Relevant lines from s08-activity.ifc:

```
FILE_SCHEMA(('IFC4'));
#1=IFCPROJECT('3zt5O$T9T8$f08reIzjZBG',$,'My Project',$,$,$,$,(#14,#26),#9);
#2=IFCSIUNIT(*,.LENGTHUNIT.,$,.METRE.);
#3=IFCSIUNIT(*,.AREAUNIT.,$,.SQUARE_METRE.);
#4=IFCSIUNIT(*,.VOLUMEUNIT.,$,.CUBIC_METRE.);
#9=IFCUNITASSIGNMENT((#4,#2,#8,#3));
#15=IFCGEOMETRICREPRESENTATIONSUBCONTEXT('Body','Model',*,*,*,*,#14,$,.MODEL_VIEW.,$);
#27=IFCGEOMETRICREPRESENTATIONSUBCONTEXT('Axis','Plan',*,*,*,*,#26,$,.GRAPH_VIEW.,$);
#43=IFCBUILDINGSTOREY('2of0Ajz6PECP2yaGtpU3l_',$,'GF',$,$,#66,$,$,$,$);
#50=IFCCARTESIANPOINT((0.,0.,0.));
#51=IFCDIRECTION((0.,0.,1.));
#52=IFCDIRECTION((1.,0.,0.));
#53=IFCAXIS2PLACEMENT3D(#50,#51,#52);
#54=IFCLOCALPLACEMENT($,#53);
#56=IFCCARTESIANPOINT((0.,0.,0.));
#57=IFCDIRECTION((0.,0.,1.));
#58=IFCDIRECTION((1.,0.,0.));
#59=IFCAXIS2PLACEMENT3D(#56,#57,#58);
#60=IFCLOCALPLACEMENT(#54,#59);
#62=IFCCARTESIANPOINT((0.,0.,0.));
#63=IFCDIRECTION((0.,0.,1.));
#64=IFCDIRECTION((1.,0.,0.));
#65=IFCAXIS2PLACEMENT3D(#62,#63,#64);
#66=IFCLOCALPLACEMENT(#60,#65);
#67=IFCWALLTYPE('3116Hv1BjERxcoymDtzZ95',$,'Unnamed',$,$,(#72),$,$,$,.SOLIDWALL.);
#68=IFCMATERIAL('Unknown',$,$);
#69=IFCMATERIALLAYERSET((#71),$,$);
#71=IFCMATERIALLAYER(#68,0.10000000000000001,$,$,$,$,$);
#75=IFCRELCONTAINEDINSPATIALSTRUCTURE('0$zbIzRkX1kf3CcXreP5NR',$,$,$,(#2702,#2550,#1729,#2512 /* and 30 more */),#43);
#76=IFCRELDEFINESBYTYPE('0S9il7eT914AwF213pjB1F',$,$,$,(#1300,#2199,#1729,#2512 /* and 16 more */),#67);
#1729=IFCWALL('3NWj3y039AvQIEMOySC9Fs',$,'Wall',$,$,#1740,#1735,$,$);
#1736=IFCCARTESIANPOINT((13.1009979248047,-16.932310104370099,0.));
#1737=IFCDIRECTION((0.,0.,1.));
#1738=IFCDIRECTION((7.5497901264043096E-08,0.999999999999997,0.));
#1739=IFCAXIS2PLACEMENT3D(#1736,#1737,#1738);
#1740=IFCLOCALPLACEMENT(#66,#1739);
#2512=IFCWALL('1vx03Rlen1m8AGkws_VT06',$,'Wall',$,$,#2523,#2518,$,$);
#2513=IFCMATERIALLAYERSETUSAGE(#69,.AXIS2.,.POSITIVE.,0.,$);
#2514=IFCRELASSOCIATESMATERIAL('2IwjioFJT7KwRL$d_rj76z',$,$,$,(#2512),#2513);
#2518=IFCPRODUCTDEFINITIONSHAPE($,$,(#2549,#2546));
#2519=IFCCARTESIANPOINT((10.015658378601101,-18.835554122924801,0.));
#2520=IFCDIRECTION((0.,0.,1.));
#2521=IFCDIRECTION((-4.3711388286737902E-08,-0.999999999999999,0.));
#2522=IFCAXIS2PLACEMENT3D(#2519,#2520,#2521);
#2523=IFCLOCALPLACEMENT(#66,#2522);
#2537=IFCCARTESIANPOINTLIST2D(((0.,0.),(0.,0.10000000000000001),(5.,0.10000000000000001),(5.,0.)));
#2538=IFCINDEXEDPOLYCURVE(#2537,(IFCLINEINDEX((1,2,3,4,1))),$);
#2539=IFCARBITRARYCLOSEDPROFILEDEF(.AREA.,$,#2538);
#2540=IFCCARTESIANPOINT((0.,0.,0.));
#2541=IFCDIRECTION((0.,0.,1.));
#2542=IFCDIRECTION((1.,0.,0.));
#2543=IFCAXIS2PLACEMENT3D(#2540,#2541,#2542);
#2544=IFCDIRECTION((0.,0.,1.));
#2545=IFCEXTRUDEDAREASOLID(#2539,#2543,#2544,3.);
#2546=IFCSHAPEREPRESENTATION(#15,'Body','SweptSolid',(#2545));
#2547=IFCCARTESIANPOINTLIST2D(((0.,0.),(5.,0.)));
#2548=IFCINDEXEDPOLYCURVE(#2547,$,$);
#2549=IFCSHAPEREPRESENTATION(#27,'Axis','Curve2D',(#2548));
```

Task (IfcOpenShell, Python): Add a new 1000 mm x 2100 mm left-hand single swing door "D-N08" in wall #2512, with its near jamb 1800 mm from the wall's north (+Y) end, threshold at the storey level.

```python
import numpy as np
import ifcopenshell
import ifcopenshell.api.feature
import ifcopenshell.api.geometry
import ifcopenshell.api.root
import ifcopenshell.api.spatial
import ifcopenshell.geom
import ifcopenshell.util.element
import ifcopenshell.util.placement
import ifcopenshell.util.representation
import ifcopenshell.util.shape
import ifcopenshell.util.unit

model = ifcopenshell.open("s08-activity.ifc")
unit_scale = ifcopenshell.util.unit.calculate_unit_scale(model)
settings = ifcopenshell.geom.settings()


def volume(element):
    """Net volume in cubic metres, openings subtracted."""
    shape = ifcopenshell.geom.create_shape(settings, element)
    return ifcopenshell.util.shape.get_volume(shape.geometry)


wall = model.by_guid("1vx03Rlen1m8AGkws_VT06")
storey = ifcopenshell.util.element.get_container(wall, ifc_class="IfcBuildingStorey")
context = ifcopenshell.util.representation.get_context(model, "Model", "Body", "MODEL_VIEW")
before = volume(wall)

width, height, from_end, sill = 1, 2.1, 1.8, 0.0  # metres

# The wall runs along its own X axis, and the end named is its -X end.
wall_shape = ifcopenshell.geom.create_shape(settings, wall)
x, y, z = ifcopenshell.util.shape.get_vertices(wall_shape.geometry).T
start = x.min() + from_end
face, thickness = float(y.min()), float(y.max() - y.min())
wall_matrix = ifcopenshell.util.placement.get_local_placement(wall.ObjectPlacement)
level = ifcopenshell.util.placement.get_local_placement(storey.ObjectPlacement)[2, 3]


def in_wall(x, y):
    """Placement at x, y metres in the wall's axes, at sill height."""
    matrix = wall_matrix.copy()
    matrix[:, 3] = wall_matrix @ np.array([x / unit_scale, y / unit_scale, 0.0, 1.0])
    matrix[2, 3] = level + sill / unit_scale
    return matrix


# Opening: a box that overshoots both wall faces by 50 mm.
opening = ifcopenshell.api.root.create_entity(model, ifc_class="IfcOpeningElement", predefined_type="OPENING")
box = ifcopenshell.api.geometry.add_wall_representation(
    model, context=context, length=width, height=height, thickness=thickness + 0.1
)
ifcopenshell.api.geometry.assign_representation(model, product=opening, representation=box)
ifcopenshell.api.geometry.edit_object_placement(model, product=opening, matrix=in_wall(start, face - 0.05), is_si=False)
ifcopenshell.api.feature.add_feature(model, feature=opening, element=wall)

door = ifcopenshell.api.root.create_entity(model, ifc_class="IfcDoor", name="D-N08", predefined_type="DOOR")
door.OverallWidth, door.OverallHeight = width / unit_scale, height / unit_scale
door.OperationType = "SINGLE_SWING_LEFT"
body = ifcopenshell.api.geometry.add_door_representation(
    model,
    context=context,
    overall_width=door.OverallWidth,
    overall_height=door.OverallHeight,
    operation_type="SINGLE_SWING_LEFT",
    lining_properties={"LiningDepth": thickness / unit_scale, "ThresholdDepth": thickness / unit_scale},
)
ifcopenshell.api.geometry.assign_representation(model, product=door, representation=body)
ifcopenshell.api.spatial.assign_container(model, products=[door], relating_structure=storey)
ifcopenshell.api.feature.add_filling(model, opening=opening, element=door)

# The lining spans the wall, so the door starts at the wall face.
ifcopenshell.api.geometry.edit_object_placement(model, product=door, matrix=in_wall(start, face), is_si=False)

after = volume(wall)

print(f"wall volume {before:.3f} -> {after:.3f} m3")

model.write("s08-activity_updated.ifc")
```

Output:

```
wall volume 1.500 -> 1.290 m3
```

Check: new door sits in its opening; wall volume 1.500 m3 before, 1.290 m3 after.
